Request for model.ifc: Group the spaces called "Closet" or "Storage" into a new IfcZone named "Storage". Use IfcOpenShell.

First a look at what the model holds.

```python
import ifcopenshell

model = ifcopenshell.open("model.ifc")
print(model.schema)
seen = {}
for space in model.by_type("IfcSpace"):
    seen[space.LongName] = seen.get(space.LongName, 0) + 1
for name, count in sorted(seen.items(), key=str):
    print(count, "x", name)
print("zones:", [z.Name for z in model.by_type("IfcZone")][:20])
```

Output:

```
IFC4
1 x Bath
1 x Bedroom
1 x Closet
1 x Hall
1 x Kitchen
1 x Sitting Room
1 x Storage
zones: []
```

```python
import ifcopenshell
import ifcopenshell.api.group
import ifcopenshell.api.root

model = ifcopenshell.open("model.ifc")

names = {"Closet", "Storage"}
spaces = [s for s in model.by_type("IfcSpace") if s.LongName in names]

zone = ifcopenshell.api.root.create_entity(model, ifc_class="IfcZone", name="Storage")
ifcopenshell.api.group.assign_group(model, products=spaces, group=zone)
print(len(spaces), "spaces in", zone.Name)

model.write("model_edited.ifc")
```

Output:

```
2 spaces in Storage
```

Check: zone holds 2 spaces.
